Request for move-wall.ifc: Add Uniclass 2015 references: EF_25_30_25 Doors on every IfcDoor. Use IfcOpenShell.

First a look at what the model holds.

```python
import ifcopenshell

model = ifcopenshell.open("move-wall.ifc")
print(model.schema)
print("classifications:", [c.Name for c in model.by_type("IfcClassification")])
for ifc_class in ("IfcDoor", "IfcRoof", "IfcStair", "IfcWall", "IfcWindow"):
    print(ifc_class, len(model.by_type(ifc_class)))
```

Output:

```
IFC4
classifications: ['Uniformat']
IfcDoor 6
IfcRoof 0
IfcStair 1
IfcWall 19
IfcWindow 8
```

```python
import ifcopenshell
import ifcopenshell.api.classification

model = ifcopenshell.open("move-wall.ifc")

system = ifcopenshell.api.classification.add_classification(model, classification="Uniclass 2015")

codes = {
    "IfcDoor": ("EF_25_30_25", "Doors"),
}
for ifc_class, (code, name) in codes.items():
    products = model.by_type(ifc_class)
    ifcopenshell.api.classification.add_reference(
        model, products=products, classification=system, identification=code, name=name
    )
    print(code, len(products))

model.write("move-wall-out.ifc")
```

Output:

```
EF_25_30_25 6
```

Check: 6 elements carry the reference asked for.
